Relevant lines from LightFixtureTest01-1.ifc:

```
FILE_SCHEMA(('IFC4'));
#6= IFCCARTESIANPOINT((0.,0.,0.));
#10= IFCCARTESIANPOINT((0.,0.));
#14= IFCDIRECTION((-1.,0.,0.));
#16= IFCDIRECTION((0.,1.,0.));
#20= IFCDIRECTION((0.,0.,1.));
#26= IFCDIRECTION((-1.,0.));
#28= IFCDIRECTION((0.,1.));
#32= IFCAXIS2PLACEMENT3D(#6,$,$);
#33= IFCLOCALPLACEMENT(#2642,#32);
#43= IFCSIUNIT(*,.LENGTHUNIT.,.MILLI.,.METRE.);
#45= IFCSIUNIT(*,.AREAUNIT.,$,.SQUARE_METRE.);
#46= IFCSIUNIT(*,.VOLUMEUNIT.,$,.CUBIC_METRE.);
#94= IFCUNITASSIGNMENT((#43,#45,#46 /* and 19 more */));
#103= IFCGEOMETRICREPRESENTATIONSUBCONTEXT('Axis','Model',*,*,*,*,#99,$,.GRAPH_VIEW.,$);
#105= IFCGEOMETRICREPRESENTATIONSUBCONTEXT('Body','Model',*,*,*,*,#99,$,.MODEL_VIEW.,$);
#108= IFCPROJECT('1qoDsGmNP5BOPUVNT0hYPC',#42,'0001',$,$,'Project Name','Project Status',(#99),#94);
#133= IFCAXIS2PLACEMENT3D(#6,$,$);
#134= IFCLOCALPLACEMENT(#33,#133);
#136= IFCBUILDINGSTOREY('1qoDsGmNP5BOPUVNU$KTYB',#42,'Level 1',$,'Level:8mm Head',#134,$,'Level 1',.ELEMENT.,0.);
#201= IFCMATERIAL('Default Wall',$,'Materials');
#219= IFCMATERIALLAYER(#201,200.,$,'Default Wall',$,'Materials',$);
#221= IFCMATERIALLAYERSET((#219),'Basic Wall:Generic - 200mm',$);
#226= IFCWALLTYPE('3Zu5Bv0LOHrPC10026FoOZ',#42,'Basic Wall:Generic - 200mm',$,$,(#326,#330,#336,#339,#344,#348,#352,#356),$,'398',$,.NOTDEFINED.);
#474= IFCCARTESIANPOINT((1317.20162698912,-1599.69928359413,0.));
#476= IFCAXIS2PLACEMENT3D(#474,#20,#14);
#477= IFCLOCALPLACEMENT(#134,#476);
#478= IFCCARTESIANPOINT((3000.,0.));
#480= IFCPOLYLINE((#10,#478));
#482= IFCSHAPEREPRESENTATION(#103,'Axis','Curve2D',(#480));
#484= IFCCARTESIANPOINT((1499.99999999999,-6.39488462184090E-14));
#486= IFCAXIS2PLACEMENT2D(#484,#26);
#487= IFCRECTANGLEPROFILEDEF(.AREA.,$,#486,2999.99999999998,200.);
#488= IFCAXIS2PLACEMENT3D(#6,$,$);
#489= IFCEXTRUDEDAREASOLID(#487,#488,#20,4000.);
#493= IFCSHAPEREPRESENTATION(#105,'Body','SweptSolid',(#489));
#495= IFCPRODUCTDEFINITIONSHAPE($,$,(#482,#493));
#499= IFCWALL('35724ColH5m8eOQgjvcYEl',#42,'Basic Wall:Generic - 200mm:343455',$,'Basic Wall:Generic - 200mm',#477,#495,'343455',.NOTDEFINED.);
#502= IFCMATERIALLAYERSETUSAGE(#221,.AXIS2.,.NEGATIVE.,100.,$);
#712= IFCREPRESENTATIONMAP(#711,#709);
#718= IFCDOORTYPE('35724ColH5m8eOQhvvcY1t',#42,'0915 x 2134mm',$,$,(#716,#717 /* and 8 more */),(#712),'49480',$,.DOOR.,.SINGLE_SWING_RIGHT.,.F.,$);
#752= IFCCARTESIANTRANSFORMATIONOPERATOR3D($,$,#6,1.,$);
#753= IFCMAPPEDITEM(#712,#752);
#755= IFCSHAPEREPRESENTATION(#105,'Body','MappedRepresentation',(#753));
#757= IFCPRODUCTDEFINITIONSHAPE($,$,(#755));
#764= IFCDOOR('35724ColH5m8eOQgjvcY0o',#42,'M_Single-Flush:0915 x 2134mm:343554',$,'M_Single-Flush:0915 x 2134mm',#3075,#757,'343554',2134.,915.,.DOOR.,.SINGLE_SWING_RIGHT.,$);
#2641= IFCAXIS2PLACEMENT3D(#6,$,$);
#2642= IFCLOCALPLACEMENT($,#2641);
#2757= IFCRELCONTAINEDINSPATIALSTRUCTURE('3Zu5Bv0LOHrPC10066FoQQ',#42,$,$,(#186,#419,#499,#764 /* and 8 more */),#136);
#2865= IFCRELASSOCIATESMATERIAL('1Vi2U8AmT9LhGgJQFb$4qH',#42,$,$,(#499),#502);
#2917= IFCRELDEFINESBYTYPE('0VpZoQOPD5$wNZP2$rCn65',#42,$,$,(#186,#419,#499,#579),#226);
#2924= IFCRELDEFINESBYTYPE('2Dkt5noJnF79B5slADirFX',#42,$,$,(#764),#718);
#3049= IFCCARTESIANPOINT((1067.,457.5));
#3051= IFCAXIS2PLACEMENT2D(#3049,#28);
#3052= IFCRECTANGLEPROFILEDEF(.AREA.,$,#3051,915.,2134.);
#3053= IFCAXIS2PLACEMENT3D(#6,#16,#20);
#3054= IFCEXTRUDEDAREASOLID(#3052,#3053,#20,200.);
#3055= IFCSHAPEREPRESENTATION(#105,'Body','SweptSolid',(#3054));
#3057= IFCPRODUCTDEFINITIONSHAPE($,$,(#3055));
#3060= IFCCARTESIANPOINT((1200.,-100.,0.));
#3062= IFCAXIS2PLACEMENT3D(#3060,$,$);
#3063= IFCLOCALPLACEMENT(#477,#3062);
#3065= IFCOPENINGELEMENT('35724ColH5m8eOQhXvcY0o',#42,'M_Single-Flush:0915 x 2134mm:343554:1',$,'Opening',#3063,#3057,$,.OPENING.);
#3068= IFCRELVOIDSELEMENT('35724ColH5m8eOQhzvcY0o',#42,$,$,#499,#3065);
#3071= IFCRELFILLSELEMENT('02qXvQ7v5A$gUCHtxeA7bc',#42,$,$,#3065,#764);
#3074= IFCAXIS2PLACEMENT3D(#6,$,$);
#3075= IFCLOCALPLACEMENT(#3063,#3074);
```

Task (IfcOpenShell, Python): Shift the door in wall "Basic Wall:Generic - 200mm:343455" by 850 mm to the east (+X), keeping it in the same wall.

```python
import ifcopenshell
import ifcopenshell.api.geometry
import ifcopenshell.util.placement

model = ifcopenshell.open("LightFixtureTest01-1.ifc")

door = model.by_guid("35724ColH5m8eOQgjvcY0o")
opening = door.FillsVoids[0].RelatingOpeningElement
wall = opening.VoidsElements[0].RelatingBuildingElement

wall_matrix = ifcopenshell.util.placement.get_local_placement(wall.ObjectPlacement)
shift = wall_matrix[:3, 0] * -850.0
before = ifcopenshell.util.placement.get_local_placement(door.ObjectPlacement)[:3, 3].copy()

# The door is placed relative to its opening, so it follows when the opening moves.
matrix = ifcopenshell.util.placement.get_local_placement(opening.ObjectPlacement)
matrix[:3, 3] += shift
ifcopenshell.api.geometry.edit_object_placement(
    model, product=opening, matrix=matrix, is_si=False, should_transform_children=True
)

after = ifcopenshell.util.placement.get_local_placement(door.ObjectPlacement)[:3, 3]
print("door moved by", (after - before).round(3) + 0.0)

model.write("LightFixtureTest01-1_updated.ifc")
```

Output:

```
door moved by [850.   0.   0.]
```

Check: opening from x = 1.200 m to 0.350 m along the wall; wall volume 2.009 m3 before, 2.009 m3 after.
